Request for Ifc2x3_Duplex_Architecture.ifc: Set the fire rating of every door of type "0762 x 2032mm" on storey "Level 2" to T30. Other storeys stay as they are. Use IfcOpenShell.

First a look at what the model holds.

```python
import ifcopenshell
import ifcopenshell.util.element

model = ifcopenshell.open("Ifc2x3_Duplex_Architecture.ifc")
print(model.schema)
storey = next(s for s in model.by_type("IfcBuildingStorey") if s.Name == "Level 2")
doors = [e for e in ifcopenshell.util.element.get_decomposition(storey) if e.is_a("IfcDoor")]
seen = {}
for e in doors:
    element_type = ifcopenshell.util.element.get_type(e)
    key = (element_type.Name if element_type != e and element_type else None, ifcopenshell.util.element.get_pset(e, "Pset_DoorCommon", "FireRating"))
    seen[key] = seen.get(key, 0) + 1
for (name, value), count in sorted(seen.items(), key=str):
    print(count, "x", name, "|", value)
```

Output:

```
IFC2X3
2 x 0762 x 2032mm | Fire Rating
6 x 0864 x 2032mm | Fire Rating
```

```python
import ifcopenshell
import ifcopenshell.api.pset
import ifcopenshell.util.element

model = ifcopenshell.open("Ifc2x3_Duplex_Architecture.ifc")

storey = next(s for s in model.by_type("IfcBuildingStorey") if s.Name == "Level 2")
doors = [e for e in ifcopenshell.util.element.get_decomposition(storey) if e.is_a("IfcDoor")]

count = 0
for e in doors:
    element_type = ifcopenshell.util.element.get_type(e)
    if element_type in (None, e) or element_type.Name != "0762 x 2032mm":
        continue
    # add_pset returns the element's existing set when there is one.
    pset = ifcopenshell.api.pset.add_pset(model, product=e, name="Pset_DoorCommon")
    ifcopenshell.api.pset.edit_pset(model, pset=pset, properties={"FireRating": "T30"})
    count += 1

print(count, "doors updated")

model.write("Ifc2x3_Duplex_Architecture_v2.ifc")
```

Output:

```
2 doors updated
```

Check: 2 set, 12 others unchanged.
